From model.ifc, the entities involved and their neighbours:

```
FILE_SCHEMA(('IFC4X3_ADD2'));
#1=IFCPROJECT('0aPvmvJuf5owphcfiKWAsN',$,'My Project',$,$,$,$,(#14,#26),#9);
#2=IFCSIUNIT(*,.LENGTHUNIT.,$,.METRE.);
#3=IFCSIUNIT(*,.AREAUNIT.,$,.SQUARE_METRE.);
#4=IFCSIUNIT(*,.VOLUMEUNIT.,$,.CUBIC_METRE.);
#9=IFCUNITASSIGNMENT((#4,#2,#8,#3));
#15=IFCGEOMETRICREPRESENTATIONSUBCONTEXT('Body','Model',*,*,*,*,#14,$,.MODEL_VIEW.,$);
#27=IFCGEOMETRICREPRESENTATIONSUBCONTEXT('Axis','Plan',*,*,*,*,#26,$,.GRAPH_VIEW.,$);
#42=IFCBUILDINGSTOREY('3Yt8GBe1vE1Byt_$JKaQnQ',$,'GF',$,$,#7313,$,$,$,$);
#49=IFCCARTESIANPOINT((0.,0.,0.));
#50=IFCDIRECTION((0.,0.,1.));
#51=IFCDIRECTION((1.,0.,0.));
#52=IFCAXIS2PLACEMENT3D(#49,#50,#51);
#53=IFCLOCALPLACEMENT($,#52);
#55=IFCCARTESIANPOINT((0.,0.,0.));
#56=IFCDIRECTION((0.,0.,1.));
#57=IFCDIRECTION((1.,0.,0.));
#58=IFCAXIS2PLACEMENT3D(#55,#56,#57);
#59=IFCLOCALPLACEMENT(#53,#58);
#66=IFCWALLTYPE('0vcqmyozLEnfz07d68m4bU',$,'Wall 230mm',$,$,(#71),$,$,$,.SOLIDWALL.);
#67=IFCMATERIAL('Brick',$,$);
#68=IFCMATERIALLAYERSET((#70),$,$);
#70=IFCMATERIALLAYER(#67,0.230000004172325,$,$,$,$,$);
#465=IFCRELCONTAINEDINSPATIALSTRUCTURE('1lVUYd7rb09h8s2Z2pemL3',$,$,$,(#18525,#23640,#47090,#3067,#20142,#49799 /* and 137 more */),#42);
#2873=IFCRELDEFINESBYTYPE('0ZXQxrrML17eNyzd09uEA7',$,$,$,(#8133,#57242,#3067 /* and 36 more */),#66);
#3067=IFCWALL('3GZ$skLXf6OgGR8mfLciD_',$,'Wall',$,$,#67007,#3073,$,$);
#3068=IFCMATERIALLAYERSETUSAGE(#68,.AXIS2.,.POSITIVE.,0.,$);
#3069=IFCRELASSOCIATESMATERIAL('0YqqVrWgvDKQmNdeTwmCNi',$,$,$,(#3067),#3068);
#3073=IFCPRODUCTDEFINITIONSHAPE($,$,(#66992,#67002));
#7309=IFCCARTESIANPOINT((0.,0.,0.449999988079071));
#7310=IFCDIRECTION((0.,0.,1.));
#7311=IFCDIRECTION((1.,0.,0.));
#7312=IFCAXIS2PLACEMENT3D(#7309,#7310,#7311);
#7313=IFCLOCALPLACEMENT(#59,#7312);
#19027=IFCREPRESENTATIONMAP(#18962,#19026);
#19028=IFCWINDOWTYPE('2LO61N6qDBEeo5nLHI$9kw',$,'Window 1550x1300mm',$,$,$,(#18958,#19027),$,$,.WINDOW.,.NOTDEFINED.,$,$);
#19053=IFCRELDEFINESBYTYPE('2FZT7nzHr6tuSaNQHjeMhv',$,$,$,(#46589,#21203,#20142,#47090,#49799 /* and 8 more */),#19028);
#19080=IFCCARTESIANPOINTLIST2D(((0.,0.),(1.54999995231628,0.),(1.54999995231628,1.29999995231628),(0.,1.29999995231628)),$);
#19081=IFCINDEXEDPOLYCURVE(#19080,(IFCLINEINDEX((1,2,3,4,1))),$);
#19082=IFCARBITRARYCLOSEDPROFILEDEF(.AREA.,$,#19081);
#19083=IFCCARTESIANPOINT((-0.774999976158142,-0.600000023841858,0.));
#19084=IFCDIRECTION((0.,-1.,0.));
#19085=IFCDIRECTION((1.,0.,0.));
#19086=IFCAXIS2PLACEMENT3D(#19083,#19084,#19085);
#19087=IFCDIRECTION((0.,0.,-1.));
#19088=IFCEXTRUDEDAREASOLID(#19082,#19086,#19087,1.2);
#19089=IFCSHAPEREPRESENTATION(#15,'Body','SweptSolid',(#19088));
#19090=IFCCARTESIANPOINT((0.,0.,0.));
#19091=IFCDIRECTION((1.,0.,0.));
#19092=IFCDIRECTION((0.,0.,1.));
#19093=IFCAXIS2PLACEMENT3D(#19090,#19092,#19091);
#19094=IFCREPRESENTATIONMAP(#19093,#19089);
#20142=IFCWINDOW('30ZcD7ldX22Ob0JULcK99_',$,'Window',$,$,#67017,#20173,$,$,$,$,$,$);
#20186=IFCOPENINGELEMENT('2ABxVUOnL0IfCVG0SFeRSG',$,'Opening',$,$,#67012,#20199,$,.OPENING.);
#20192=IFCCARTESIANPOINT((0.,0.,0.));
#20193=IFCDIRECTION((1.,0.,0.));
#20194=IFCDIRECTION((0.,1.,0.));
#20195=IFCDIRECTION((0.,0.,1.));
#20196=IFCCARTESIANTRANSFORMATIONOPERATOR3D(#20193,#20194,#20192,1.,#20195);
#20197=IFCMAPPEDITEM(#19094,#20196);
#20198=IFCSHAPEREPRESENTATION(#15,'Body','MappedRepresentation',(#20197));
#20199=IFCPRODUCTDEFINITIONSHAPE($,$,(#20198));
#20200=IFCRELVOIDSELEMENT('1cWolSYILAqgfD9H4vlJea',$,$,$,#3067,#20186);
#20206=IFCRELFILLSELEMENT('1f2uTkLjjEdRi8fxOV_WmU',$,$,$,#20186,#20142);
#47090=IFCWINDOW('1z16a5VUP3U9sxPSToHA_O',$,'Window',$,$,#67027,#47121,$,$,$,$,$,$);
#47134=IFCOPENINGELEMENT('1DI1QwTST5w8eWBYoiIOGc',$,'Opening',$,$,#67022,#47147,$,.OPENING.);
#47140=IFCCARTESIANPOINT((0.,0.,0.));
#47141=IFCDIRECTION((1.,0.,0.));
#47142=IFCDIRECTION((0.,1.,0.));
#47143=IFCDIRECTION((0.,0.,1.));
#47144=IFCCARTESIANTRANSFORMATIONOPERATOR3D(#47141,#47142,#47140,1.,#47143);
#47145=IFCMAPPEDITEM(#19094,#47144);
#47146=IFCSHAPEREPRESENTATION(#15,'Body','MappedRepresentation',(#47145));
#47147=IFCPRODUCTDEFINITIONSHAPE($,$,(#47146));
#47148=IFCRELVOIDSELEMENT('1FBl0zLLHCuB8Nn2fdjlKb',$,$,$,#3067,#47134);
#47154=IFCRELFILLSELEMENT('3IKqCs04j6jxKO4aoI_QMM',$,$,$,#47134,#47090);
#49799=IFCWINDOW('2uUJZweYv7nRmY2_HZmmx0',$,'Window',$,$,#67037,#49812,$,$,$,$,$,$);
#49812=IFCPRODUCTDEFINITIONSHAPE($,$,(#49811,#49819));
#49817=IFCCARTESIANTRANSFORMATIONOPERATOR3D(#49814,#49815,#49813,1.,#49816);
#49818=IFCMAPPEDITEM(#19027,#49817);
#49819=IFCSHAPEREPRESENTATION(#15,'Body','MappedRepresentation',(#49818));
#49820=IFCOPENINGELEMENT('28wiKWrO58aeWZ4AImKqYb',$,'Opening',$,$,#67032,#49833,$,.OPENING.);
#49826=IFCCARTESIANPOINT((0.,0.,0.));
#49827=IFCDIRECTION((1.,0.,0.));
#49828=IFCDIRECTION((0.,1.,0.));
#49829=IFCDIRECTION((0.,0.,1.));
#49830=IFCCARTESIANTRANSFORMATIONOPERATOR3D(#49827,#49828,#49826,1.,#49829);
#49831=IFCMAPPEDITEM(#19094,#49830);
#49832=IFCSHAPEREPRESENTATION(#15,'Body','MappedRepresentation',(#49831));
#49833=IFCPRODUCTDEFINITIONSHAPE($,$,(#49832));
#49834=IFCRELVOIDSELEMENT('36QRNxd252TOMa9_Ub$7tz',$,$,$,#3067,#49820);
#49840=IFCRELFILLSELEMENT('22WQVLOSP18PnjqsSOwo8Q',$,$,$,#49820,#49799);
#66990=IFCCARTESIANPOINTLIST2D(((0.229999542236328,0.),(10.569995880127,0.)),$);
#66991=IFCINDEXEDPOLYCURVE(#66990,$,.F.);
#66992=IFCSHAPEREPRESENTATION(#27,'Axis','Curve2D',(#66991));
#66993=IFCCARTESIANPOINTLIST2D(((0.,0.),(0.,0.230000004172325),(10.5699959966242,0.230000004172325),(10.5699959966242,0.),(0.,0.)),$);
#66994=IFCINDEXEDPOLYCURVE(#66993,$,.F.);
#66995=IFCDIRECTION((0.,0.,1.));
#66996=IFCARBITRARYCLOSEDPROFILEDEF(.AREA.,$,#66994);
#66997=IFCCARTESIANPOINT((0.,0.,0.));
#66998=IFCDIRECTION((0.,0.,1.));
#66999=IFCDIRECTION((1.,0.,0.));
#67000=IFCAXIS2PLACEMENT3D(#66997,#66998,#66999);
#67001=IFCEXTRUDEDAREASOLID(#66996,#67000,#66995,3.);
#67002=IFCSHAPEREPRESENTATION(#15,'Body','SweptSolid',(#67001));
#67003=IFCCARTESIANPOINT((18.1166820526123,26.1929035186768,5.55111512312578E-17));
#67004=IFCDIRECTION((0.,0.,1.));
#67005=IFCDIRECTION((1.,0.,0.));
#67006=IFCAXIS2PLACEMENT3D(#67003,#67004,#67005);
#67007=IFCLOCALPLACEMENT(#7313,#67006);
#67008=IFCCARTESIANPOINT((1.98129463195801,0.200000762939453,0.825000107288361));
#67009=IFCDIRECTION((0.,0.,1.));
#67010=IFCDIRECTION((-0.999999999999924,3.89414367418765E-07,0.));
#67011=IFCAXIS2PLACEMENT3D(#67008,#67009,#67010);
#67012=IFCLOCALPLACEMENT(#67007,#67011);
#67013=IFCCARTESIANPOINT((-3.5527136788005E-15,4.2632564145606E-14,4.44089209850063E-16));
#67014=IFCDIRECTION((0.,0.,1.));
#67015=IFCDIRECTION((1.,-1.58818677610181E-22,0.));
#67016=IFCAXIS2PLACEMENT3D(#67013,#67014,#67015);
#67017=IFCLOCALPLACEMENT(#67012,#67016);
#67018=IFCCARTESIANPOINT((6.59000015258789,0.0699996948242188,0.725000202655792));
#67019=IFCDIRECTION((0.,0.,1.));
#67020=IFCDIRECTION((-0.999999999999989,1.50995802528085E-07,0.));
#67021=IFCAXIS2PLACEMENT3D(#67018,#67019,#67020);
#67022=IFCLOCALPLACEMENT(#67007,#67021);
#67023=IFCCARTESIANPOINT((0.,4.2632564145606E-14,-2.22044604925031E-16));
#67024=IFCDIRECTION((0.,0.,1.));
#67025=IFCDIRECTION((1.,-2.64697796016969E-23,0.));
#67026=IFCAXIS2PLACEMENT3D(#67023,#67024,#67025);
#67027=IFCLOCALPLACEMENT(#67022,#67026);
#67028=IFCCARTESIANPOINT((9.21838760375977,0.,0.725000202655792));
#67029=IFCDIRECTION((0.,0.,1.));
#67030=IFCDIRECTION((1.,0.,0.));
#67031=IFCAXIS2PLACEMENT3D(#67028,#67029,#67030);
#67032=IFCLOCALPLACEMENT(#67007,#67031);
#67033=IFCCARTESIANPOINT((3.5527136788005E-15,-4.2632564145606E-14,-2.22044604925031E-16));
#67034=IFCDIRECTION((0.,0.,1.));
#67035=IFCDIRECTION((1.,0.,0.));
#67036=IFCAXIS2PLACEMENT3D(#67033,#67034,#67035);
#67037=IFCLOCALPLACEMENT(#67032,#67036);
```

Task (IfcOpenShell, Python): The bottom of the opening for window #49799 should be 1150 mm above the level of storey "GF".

```python
import numpy as np
import ifcopenshell
import ifcopenshell.api.geometry
import ifcopenshell.geom
import ifcopenshell.util.element
import ifcopenshell.util.placement
import ifcopenshell.util.shape
import ifcopenshell.util.unit

model = ifcopenshell.open("model.ifc")
unit_scale = ifcopenshell.util.unit.calculate_unit_scale(model)

window = model.by_id(49799)
opening = window.FillsVoids[0].RelatingOpeningElement
storey = ifcopenshell.util.element.get_container(window, ifc_class="IfcBuildingStorey")
level = ifcopenshell.util.placement.get_local_placement(storey.ObjectPlacement)[2, 3]

# The opening's origin need not be at the sill, so measure its lowest point.
shape = ifcopenshell.geom.create_shape(ifcopenshell.geom.settings(), opening)
bottom = ifcopenshell.util.shape.get_shape_bottom_elevation(shape, shape.geometry) / unit_scale
dz = level + 1.15 / unit_scale - bottom

shift = np.array([0.0, 0.0, dz])
# The window is placed relative to its opening, so it follows when the opening moves.
matrix = ifcopenshell.util.placement.get_local_placement(opening.ObjectPlacement)
matrix[:3, 3] += shift
ifcopenshell.api.geometry.edit_object_placement(
    model, product=opening, matrix=matrix, is_si=False, should_transform_children=True
)

print(f"moved by {dz * unit_scale:+.3f} m")

model.write("model_edited.ifc")
```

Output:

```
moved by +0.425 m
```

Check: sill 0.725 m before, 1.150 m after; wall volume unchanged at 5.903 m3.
